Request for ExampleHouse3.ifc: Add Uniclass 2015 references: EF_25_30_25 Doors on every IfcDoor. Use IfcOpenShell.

First a look at what the model holds.

```python
import ifcopenshell

model = ifcopenshell.open("ExampleHouse3.ifc")
print(model.schema)
print("classifications:", [c.Name for c in model.by_type("IfcClassification")])
for ifc_class in ("IfcDoor", "IfcRoof", "IfcStair", "IfcWall", "IfcWindow"):
    print(ifc_class, len(model.by_type(ifc_class)))
```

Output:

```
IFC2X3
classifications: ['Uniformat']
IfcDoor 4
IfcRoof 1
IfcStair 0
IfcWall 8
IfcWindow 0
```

```python
import ifcopenshell
import ifcopenshell.api.classification

model = ifcopenshell.open("ExampleHouse3.ifc")

# IFC2X3 requires Source and Edition and has no link from the project to the system.
system = model.create_entity("IfcClassification", Source="NBS", Edition="2015", Name="Uniclass 2015")

codes = {
    "IfcDoor": ("EF_25_30_25", "Doors"),
}
for ifc_class, (code, name) in codes.items():
    products = model.by_type(ifc_class)
    ifcopenshell.api.classification.add_reference(
        model, products=products, classification=system, identification=code, name=name
    )
    print(code, len(products))

model.write("ExampleHouse3_edited.ifc")
```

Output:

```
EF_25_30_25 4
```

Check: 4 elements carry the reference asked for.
